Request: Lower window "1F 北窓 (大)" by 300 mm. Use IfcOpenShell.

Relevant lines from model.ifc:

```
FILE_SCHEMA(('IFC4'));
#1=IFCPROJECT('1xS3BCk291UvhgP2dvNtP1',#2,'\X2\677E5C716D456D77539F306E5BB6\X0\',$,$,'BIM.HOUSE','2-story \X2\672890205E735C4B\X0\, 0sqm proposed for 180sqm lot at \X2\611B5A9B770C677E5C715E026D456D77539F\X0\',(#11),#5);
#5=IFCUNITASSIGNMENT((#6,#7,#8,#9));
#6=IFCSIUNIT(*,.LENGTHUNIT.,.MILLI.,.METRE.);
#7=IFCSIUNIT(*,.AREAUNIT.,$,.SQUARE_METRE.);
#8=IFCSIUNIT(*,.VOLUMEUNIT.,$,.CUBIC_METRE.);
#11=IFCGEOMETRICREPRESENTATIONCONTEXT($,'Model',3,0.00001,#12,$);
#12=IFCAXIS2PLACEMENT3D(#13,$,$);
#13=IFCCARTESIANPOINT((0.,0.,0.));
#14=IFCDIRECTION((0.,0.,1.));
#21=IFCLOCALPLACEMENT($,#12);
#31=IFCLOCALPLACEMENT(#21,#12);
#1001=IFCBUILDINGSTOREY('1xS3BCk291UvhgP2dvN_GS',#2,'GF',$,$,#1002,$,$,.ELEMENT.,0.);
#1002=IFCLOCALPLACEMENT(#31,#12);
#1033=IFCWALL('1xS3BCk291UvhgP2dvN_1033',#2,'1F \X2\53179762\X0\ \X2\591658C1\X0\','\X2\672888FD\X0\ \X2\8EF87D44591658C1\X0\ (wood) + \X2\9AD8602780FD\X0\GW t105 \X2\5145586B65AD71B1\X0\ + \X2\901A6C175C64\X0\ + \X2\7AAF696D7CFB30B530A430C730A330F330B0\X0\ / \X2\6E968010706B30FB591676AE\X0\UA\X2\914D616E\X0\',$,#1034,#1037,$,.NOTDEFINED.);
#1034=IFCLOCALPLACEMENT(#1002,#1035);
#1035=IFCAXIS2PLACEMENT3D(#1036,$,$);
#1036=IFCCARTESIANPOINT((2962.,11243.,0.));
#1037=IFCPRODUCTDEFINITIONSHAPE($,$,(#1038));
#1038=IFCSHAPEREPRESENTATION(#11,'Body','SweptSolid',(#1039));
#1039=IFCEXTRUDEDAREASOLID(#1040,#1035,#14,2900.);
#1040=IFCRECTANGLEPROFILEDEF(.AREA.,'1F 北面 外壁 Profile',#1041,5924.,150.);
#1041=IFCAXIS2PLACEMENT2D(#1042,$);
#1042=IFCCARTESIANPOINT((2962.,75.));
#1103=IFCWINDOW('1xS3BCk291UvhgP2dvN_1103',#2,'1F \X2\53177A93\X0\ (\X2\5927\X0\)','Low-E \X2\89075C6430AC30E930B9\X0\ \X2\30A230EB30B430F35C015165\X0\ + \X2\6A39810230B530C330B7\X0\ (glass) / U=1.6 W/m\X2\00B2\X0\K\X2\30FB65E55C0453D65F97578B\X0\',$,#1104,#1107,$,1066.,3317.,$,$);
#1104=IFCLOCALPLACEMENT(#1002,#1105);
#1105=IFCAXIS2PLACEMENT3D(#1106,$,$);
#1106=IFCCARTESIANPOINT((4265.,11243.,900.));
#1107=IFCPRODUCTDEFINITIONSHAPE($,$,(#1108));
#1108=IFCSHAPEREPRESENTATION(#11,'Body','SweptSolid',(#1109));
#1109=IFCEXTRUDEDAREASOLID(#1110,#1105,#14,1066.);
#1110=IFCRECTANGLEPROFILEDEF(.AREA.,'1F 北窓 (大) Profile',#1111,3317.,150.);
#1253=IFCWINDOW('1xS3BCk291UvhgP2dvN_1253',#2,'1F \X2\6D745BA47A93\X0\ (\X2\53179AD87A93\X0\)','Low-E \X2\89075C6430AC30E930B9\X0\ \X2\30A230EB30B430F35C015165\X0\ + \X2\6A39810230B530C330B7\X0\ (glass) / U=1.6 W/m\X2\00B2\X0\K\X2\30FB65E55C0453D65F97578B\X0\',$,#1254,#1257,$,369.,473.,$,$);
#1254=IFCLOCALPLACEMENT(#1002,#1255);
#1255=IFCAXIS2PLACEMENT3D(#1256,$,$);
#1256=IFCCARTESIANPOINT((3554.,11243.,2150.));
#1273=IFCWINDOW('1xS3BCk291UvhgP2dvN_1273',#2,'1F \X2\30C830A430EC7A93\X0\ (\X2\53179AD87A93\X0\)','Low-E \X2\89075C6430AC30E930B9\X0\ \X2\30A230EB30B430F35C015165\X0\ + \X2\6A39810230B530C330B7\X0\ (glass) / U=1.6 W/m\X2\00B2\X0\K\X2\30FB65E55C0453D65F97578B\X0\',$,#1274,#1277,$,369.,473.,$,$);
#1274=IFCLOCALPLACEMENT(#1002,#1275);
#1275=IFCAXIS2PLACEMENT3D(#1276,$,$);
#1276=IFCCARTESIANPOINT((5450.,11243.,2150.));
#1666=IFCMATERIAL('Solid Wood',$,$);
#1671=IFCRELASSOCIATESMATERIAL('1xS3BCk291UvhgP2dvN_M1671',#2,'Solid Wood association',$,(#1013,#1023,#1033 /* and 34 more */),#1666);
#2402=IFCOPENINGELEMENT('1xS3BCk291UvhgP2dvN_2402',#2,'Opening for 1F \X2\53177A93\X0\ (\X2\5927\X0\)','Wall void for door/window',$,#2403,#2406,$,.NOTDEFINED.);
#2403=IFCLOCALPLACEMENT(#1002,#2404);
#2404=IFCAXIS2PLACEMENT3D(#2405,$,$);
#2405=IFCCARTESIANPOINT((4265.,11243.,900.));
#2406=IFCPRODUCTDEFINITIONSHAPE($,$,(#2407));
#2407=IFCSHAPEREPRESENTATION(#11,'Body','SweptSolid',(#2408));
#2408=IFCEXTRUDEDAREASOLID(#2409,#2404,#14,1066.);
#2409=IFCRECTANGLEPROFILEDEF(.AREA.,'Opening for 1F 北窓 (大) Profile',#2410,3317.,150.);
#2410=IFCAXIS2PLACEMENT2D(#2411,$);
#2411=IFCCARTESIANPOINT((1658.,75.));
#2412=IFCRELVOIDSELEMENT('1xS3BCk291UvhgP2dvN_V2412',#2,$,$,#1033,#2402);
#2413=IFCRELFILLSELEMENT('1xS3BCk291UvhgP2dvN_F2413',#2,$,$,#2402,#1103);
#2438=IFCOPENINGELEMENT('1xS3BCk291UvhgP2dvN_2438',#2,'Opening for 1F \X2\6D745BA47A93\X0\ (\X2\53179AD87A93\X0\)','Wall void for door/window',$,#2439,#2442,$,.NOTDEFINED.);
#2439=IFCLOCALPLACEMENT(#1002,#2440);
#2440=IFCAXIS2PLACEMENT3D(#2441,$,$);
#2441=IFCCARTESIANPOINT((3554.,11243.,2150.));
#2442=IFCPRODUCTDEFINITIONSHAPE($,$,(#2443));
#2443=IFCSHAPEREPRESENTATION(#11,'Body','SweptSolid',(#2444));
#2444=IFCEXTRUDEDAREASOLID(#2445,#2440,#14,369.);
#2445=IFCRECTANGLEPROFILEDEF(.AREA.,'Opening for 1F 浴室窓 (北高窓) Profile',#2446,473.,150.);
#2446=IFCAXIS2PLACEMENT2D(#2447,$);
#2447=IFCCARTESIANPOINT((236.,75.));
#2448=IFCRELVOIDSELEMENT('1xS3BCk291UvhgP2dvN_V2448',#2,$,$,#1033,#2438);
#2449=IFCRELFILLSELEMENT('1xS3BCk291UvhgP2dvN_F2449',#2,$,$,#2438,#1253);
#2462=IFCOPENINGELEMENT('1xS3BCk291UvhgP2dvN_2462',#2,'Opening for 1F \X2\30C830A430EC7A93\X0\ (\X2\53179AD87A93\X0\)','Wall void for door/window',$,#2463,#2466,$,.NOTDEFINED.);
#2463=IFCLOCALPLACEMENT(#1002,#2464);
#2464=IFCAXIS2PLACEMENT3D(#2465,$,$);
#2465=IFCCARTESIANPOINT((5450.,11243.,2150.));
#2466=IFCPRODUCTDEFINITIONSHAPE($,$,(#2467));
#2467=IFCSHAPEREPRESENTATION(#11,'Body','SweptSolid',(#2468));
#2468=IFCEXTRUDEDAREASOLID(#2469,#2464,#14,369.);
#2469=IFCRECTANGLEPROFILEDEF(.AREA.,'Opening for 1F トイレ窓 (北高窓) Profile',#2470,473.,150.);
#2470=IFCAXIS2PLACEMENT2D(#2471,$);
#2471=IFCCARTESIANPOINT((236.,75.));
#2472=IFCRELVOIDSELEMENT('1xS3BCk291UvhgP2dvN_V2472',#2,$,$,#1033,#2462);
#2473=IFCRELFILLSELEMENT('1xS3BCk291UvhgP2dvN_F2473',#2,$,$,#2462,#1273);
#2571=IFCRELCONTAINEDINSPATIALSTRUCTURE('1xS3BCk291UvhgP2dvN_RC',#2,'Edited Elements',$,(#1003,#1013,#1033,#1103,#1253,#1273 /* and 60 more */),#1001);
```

```python
import numpy as np
import ifcopenshell
import ifcopenshell.api.geometry
import ifcopenshell.util.placement
import ifcopenshell.util.unit

model = ifcopenshell.open("model.ifc")
unit_scale = ifcopenshell.util.unit.calculate_unit_scale(model)

window = model.by_guid("1xS3BCk291UvhgP2dvN_1103")
opening = window.FillsVoids[0].RelatingOpeningElement
dz = -300.0

shift = np.array([0.0, 0.0, dz])
# The window is not placed relative to its opening, so move both.
for product in (opening, window):
    matrix = ifcopenshell.util.placement.get_local_placement(product.ObjectPlacement)
    matrix[:3, 3] += shift
    ifcopenshell.api.geometry.edit_object_placement(model, product=product, matrix=matrix, is_si=False)

print(f"moved by {dz * unit_scale:+.3f} m")

model.write("model_updated.ifc")
```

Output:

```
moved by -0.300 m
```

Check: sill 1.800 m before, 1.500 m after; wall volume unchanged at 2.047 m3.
